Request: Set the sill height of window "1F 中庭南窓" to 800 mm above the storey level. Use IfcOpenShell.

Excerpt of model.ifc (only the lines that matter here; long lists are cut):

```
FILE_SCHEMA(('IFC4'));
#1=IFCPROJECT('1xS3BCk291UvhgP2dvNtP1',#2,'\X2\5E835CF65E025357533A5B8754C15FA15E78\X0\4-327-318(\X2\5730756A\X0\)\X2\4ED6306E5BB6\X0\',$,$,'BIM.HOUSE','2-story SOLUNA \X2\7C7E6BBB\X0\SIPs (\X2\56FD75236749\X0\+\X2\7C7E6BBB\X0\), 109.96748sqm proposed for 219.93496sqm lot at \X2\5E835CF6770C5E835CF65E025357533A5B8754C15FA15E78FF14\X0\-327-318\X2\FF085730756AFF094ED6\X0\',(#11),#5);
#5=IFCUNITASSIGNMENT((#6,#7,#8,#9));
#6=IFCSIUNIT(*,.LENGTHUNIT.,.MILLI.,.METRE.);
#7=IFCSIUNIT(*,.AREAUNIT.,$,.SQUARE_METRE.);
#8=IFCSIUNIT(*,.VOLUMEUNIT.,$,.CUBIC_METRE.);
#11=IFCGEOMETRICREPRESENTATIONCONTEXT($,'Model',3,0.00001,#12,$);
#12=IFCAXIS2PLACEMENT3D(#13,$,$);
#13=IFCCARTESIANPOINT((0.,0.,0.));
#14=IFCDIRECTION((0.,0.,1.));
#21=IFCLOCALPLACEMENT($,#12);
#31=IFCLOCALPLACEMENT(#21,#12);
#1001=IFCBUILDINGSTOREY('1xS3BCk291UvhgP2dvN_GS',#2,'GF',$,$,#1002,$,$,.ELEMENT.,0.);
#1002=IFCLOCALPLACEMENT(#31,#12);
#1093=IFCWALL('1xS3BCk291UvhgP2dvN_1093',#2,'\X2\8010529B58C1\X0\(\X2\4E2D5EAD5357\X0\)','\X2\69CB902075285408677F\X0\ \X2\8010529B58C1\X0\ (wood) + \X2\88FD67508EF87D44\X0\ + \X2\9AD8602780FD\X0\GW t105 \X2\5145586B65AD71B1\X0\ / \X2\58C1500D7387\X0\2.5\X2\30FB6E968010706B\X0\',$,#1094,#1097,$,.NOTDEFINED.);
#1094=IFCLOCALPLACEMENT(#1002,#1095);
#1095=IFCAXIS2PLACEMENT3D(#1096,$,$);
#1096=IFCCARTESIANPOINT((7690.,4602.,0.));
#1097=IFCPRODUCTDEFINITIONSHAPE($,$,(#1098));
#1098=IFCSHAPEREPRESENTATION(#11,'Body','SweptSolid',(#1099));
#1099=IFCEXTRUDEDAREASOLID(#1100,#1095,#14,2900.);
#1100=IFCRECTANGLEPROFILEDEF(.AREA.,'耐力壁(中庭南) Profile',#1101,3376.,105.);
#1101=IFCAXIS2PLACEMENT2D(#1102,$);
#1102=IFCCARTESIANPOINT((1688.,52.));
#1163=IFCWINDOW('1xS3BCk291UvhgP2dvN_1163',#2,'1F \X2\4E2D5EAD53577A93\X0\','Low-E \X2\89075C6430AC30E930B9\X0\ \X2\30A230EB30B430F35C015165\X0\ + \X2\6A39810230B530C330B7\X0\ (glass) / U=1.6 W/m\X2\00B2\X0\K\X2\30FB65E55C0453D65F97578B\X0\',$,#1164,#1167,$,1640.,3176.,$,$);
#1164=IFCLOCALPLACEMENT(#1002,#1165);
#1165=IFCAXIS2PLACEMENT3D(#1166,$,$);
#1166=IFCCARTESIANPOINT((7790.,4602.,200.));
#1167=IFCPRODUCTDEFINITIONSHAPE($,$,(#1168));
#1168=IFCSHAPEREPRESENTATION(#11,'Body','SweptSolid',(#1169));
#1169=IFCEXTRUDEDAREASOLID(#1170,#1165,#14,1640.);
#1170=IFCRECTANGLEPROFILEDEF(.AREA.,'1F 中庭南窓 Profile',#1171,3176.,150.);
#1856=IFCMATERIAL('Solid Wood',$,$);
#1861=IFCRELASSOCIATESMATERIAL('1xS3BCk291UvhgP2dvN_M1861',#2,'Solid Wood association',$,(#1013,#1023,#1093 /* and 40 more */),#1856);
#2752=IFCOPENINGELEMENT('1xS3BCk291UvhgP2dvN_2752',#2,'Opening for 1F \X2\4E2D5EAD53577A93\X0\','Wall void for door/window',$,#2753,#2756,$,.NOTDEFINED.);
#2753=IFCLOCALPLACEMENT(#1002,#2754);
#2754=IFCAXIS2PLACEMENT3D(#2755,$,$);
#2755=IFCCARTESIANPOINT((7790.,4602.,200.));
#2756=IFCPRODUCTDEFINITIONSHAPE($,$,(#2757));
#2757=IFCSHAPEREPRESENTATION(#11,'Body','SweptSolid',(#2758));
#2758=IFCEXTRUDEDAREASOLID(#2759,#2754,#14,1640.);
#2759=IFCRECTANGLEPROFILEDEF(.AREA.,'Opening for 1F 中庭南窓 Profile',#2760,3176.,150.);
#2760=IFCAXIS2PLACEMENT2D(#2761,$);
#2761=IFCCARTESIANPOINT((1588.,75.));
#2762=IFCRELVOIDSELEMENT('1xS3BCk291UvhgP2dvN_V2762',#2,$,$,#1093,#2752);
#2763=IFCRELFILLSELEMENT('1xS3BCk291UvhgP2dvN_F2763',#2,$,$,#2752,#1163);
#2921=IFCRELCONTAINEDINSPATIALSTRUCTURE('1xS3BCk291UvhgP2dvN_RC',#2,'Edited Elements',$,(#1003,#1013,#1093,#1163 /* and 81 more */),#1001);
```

```python
import numpy as np
import ifcopenshell
import ifcopenshell.api.geometry
import ifcopenshell.geom
import ifcopenshell.util.element
import ifcopenshell.util.placement
import ifcopenshell.util.shape
import ifcopenshell.util.unit

model = ifcopenshell.open("model.ifc")
unit_scale = ifcopenshell.util.unit.calculate_unit_scale(model)

window = model.by_guid("1xS3BCk291UvhgP2dvN_1163")
opening = window.FillsVoids[0].RelatingOpeningElement
storey = ifcopenshell.util.element.get_container(window, ifc_class="IfcBuildingStorey")
level = ifcopenshell.util.placement.get_local_placement(storey.ObjectPlacement)[2, 3]

# The opening's origin need not be at the sill, so measure its lowest point.
shape = ifcopenshell.geom.create_shape(ifcopenshell.geom.settings(), opening)
bottom = ifcopenshell.util.shape.get_shape_bottom_elevation(shape, shape.geometry) / unit_scale
dz = level + 800.0 - bottom

shift = np.array([0.0, 0.0, dz])
# The window is not placed relative to its opening, so move both.
for product in (opening, window):
    matrix = ifcopenshell.util.placement.get_local_placement(product.ObjectPlacement)
    matrix[:3, 3] += shift
    ifcopenshell.api.geometry.edit_object_placement(model, product=product, matrix=matrix, is_si=False)

print(f"moved by {dz * unit_scale:+.3f} m")

model.write("model-out.ifc")
```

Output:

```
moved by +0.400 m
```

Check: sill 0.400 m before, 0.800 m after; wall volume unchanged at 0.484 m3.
